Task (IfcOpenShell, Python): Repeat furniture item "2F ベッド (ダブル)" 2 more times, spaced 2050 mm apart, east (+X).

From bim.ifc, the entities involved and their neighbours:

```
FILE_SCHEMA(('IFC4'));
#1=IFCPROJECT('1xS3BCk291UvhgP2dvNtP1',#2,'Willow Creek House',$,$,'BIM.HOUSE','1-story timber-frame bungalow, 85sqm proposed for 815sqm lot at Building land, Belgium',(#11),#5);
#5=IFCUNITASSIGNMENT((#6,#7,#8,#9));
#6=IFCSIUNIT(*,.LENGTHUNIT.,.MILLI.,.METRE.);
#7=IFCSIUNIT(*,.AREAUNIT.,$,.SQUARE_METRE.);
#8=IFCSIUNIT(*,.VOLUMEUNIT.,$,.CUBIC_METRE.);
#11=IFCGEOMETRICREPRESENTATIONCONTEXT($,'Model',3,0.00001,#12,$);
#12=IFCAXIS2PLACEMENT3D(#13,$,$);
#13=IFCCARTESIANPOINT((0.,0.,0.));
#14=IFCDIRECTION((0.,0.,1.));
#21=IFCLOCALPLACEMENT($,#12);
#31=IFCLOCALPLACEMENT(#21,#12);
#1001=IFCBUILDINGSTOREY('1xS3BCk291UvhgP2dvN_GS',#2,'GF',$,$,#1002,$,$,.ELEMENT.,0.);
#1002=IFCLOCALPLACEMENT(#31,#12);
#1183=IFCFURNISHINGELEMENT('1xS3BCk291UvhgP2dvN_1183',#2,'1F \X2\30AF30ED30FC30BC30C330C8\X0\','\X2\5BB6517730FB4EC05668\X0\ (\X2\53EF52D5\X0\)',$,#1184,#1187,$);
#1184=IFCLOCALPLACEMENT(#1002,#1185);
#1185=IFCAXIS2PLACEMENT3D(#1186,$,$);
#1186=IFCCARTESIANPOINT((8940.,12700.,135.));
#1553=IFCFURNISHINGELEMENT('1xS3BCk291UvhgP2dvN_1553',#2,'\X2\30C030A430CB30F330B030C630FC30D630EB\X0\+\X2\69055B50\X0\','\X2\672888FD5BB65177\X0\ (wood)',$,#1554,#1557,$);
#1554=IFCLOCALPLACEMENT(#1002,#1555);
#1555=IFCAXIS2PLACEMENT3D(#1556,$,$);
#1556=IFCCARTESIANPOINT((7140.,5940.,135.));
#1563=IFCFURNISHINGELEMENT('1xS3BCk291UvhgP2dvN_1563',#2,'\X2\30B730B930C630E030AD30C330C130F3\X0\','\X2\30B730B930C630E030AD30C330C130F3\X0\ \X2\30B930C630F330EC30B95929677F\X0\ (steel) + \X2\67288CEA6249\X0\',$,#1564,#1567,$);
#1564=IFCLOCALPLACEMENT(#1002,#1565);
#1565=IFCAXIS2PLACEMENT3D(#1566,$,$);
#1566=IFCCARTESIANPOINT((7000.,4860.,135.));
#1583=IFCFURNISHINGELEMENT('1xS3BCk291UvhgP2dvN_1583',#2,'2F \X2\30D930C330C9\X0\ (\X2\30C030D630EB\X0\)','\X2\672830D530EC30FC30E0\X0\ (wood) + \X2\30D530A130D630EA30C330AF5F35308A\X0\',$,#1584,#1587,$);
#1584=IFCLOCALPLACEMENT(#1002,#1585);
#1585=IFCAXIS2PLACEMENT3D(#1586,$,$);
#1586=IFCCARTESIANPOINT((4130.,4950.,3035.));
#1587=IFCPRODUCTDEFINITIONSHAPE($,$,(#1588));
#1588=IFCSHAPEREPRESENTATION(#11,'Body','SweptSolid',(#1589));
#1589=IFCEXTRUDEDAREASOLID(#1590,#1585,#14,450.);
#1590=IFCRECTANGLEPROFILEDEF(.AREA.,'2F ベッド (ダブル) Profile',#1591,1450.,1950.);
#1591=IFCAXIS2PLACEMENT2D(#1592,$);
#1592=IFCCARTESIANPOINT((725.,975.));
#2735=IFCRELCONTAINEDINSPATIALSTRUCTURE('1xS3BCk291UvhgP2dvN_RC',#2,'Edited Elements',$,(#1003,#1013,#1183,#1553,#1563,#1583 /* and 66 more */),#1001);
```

```python
import numpy as np
import ifcopenshell
import ifcopenshell.api.geometry
import ifcopenshell.api.root
import ifcopenshell.util.element
import ifcopenshell.util.placement
import ifcopenshell.util.unit

model = ifcopenshell.open("bim.ifc")
unit_scale = ifcopenshell.util.unit.calculate_unit_scale(model)


def reuse_history(source, copy):
    """copy_class also copies each property set's owner history, people and application; keep the originals."""
    for rel in copy.IsDefinedBy:
        if rel.is_a("IfcRelDefinesByProperties") and (history := rel.RelatingPropertyDefinition.OwnerHistory):
            rel.RelatingPropertyDefinition.OwnerHistory = source.OwnerHistory
            ifcopenshell.util.element.remove_deep2(model, history)


source = model.by_id(1583)
base = ifcopenshell.util.placement.get_local_placement(source.ObjectPlacement)
step = np.array([1.0, 0.0, 0.0]) * 2.05 / unit_scale

for i in range(1, 3):
    copy = ifcopenshell.api.root.copy_class(model, product=source)
    copy.Representation = ifcopenshell.util.element.copy_deep(
        model, source.Representation, exclude=["IfcGeometricRepresentationContext", "IfcRepresentationMap"]
    )
    reuse_history(source, copy)
    matrix = base.copy()
    matrix[:3, 3] += i * step
    print("added at", matrix[:3, 3].round(3) + 0.0)
    ifcopenshell.api.geometry.edit_object_placement(model, product=copy, matrix=matrix, is_si=False)

model.write("bim_edited.ifc")
```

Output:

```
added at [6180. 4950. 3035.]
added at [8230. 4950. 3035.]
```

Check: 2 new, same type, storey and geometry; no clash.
